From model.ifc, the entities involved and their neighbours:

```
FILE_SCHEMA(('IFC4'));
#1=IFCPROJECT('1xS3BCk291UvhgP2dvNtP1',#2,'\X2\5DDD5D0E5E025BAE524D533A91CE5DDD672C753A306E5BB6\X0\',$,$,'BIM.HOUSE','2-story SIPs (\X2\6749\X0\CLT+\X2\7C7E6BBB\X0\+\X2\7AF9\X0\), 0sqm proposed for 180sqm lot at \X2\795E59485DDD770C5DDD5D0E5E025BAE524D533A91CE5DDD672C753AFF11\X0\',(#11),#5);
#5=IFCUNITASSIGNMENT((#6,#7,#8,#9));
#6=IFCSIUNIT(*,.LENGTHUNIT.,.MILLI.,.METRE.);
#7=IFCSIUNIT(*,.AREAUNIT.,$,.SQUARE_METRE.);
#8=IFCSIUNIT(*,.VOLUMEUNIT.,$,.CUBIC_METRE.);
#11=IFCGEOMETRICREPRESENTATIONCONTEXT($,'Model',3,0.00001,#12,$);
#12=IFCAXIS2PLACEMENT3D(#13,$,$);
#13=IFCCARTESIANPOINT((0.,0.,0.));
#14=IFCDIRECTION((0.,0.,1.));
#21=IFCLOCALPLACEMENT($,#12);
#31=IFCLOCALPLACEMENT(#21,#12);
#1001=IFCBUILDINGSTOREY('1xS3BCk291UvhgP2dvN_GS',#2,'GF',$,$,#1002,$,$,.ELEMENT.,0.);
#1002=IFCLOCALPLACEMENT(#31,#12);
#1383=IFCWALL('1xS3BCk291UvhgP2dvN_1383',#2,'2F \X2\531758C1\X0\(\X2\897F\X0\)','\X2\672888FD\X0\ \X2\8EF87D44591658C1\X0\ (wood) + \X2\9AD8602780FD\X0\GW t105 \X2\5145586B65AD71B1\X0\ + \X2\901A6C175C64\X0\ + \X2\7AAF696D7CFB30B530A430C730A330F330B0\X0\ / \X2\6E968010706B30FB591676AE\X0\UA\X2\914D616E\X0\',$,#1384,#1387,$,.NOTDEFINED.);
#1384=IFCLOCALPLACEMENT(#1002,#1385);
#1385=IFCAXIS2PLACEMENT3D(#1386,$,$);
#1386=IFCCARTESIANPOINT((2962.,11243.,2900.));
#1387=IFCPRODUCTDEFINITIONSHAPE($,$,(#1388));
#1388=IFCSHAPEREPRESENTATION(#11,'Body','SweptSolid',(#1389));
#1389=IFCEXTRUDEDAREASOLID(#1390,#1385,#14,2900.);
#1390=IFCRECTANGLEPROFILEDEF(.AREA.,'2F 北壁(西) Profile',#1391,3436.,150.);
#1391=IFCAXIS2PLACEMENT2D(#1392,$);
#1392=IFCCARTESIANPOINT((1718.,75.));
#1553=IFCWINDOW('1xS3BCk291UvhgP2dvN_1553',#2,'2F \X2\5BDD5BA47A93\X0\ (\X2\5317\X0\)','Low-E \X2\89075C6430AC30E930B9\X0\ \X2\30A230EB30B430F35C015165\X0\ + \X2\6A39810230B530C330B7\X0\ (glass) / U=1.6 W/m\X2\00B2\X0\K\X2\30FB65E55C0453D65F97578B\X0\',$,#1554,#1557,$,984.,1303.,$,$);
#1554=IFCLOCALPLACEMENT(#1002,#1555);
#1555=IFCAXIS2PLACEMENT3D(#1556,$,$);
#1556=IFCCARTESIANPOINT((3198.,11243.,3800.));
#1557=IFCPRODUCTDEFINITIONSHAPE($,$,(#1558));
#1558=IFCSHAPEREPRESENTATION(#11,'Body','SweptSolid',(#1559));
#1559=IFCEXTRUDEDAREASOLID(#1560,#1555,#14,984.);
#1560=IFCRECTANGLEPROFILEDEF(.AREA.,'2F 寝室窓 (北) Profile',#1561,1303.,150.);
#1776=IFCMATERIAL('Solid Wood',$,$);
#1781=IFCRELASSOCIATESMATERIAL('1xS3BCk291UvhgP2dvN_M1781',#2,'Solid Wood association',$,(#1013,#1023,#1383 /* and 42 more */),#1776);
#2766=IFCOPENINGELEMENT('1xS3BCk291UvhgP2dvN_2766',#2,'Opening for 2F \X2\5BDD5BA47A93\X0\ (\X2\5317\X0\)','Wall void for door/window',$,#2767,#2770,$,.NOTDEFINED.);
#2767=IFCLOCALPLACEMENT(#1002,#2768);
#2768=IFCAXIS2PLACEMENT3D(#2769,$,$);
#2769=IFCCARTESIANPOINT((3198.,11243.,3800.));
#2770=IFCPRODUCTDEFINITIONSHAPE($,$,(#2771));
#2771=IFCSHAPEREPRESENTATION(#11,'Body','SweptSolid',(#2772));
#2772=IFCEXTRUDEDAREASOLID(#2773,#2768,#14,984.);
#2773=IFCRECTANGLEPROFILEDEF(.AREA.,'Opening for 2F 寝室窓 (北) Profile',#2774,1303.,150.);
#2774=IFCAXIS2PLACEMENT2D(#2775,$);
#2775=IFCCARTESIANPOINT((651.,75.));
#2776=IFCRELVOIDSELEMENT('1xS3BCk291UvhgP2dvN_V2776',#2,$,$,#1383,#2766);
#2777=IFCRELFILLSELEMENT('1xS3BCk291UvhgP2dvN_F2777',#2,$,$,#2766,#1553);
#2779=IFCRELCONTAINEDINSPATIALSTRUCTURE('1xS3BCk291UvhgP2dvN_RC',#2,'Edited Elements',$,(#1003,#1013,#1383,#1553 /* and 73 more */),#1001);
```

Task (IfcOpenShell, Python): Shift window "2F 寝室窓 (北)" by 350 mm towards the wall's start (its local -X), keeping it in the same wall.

```python
import ifcopenshell
import ifcopenshell.api.geometry
import ifcopenshell.util.placement
import ifcopenshell.util.unit

model = ifcopenshell.open("model.ifc")
unit_scale = ifcopenshell.util.unit.calculate_unit_scale(model)

window = model.by_id(1553)
opening = window.FillsVoids[0].RelatingOpeningElement
wall = opening.VoidsElements[0].RelatingBuildingElement

wall_matrix = ifcopenshell.util.placement.get_local_placement(wall.ObjectPlacement)
shift = wall_matrix[:3, 0] * -0.35 / unit_scale
before = ifcopenshell.util.placement.get_local_placement(window.ObjectPlacement)[:3, 3].copy()

# The window is not placed relative to its opening, so move both.
for product in (opening, window):
    matrix = ifcopenshell.util.placement.get_local_placement(product.ObjectPlacement)
    matrix[:3, 3] += shift
    ifcopenshell.api.geometry.edit_object_placement(model, product=product, matrix=matrix, is_si=False)

after = ifcopenshell.util.placement.get_local_placement(window.ObjectPlacement)[:3, 3]
print("window moved by", (after - before).round(3) + 0.0)

model.write("model-out.ifc")
```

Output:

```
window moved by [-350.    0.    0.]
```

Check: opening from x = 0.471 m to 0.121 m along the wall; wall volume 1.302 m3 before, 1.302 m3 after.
